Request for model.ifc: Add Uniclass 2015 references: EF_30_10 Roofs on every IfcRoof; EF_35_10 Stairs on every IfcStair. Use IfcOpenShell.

First a look at what the model holds.

```python
import ifcopenshell

model = ifcopenshell.open("model.ifc")
print(model.schema)
print("classifications:", [c.Name for c in model.by_type("IfcClassification")])
for ifc_class in ("IfcDoor", "IfcRoof", "IfcStair", "IfcWall", "IfcWindow"):
    print(ifc_class, len(model.by_type(ifc_class)))
```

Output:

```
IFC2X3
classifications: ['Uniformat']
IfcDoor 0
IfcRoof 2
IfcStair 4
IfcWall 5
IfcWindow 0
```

```python
import ifcopenshell
import ifcopenshell.api.classification

model = ifcopenshell.open("model.ifc")

# IFC2X3 requires Source and Edition and has no link from the project to the system.
system = model.create_entity("IfcClassification", Source="NBS", Edition="2015", Name="Uniclass 2015")

codes = {
    "IfcRoof": ("EF_30_10", "Roofs"),
    "IfcStair": ("EF_35_10", "Stairs"),
}
for ifc_class, (code, name) in codes.items():
    products = model.by_type(ifc_class)
    ifcopenshell.api.classification.add_reference(
        model, products=products, classification=system, identification=code, name=name
    )
    print(code, len(products))

model.write("model_edited.ifc")
```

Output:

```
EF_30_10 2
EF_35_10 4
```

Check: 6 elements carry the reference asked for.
